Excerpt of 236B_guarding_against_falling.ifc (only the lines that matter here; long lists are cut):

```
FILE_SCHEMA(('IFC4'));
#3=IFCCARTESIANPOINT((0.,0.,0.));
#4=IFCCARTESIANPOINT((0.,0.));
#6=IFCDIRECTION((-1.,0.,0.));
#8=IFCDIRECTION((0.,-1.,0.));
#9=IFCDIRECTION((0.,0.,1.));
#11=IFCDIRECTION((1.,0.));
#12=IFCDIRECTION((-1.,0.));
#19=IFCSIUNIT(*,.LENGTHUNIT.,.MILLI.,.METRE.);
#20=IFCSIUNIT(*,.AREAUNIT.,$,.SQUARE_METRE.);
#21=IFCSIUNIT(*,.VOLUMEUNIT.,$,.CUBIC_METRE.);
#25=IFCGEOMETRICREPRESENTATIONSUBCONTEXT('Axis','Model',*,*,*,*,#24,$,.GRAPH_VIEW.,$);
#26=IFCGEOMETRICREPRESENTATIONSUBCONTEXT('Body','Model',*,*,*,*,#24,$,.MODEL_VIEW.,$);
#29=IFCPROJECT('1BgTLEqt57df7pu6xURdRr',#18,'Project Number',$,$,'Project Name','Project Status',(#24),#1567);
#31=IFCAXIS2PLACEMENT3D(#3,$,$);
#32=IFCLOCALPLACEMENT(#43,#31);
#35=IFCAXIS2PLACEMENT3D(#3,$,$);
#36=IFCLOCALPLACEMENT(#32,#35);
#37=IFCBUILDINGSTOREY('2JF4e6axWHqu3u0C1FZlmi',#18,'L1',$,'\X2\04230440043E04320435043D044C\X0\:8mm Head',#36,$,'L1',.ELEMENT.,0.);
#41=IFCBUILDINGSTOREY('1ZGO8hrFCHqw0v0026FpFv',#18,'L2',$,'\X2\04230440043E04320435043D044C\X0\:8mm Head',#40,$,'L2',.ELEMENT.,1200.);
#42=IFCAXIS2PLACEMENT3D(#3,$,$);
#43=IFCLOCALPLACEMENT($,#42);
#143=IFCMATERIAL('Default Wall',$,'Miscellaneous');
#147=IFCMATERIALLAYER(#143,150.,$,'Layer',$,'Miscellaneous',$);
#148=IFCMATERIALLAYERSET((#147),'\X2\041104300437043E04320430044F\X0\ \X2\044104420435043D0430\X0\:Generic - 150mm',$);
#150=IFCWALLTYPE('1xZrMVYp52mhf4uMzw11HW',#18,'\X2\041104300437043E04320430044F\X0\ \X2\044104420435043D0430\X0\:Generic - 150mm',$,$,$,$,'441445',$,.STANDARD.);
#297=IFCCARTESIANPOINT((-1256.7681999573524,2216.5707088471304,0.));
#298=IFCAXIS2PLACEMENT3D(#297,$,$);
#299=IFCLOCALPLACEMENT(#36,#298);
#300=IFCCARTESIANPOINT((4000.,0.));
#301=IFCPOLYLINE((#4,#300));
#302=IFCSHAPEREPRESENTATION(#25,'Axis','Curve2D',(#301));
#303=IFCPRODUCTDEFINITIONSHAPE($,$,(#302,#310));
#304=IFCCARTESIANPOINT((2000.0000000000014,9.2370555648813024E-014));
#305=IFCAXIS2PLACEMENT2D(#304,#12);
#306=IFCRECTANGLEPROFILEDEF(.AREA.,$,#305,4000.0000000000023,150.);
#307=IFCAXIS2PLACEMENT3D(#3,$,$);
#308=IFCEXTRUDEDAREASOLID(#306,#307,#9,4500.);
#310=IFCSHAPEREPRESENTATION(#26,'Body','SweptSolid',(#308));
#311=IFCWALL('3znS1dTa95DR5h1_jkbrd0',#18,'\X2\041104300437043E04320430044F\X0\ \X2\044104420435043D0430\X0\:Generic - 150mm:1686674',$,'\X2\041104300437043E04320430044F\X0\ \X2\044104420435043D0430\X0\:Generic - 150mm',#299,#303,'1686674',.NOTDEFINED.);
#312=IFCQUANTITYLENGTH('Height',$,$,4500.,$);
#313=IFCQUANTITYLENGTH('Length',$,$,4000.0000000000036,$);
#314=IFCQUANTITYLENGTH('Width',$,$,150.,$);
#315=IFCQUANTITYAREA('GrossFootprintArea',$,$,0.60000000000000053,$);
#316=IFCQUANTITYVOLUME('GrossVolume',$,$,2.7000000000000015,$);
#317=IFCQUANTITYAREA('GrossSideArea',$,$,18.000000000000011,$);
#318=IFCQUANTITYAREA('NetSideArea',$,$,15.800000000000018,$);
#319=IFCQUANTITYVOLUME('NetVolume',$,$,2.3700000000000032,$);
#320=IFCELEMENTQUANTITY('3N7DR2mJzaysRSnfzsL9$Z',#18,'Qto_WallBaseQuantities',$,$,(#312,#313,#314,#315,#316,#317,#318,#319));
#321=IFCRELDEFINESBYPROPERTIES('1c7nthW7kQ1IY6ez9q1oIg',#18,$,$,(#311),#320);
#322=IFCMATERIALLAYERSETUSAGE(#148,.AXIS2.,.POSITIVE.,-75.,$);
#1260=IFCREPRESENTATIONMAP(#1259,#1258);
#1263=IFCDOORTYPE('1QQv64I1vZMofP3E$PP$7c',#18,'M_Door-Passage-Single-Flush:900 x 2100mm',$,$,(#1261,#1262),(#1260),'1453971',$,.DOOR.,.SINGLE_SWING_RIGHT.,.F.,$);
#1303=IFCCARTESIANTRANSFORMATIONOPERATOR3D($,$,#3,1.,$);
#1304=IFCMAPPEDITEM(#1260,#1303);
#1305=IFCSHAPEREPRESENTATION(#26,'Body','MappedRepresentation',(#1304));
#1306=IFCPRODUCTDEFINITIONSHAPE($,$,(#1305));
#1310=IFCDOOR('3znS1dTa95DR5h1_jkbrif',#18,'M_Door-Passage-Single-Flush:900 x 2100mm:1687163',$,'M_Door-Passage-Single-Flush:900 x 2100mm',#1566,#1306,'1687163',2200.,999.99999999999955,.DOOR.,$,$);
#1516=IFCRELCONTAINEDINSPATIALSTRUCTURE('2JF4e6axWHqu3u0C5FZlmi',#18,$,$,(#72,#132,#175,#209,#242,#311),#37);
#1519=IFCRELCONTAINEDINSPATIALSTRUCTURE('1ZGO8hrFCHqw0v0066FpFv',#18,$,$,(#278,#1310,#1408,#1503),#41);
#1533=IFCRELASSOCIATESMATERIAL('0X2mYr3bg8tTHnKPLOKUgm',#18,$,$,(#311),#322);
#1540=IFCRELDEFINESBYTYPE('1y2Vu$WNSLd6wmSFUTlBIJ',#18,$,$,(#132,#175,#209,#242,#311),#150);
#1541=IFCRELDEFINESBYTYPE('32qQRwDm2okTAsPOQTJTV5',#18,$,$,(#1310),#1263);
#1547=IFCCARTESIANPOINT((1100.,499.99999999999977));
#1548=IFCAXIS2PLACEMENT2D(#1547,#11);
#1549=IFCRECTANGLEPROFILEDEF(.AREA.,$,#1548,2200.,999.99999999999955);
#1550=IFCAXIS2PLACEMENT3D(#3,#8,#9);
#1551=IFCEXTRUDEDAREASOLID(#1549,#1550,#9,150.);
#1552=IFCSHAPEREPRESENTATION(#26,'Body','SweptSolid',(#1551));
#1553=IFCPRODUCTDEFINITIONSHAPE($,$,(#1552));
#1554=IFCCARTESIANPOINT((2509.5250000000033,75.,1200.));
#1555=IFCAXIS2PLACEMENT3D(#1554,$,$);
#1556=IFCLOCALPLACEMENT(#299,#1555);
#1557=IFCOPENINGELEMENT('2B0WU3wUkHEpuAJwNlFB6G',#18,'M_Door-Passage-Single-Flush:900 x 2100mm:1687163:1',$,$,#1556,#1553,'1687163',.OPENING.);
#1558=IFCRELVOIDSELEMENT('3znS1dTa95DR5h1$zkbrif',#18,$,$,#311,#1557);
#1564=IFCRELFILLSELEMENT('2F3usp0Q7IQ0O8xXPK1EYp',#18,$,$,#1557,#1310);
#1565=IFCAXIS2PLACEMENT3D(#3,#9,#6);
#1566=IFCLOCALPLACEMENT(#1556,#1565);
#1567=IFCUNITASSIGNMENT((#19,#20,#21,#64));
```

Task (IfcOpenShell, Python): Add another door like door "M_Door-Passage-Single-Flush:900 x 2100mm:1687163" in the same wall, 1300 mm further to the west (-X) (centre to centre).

```python
import ifcopenshell
import ifcopenshell.api.feature
import ifcopenshell.api.geometry
import ifcopenshell.api.pset
import ifcopenshell.api.root
import ifcopenshell.geom
import ifcopenshell.util.element
import ifcopenshell.util.placement
import ifcopenshell.util.shape
import ifcopenshell.util.unit

model = ifcopenshell.open("236B_guarding_against_falling.ifc")
area_scale = ifcopenshell.util.unit.calculate_unit_scale(model, "AREAUNIT")
volume_scale = ifcopenshell.util.unit.calculate_unit_scale(model, "VOLUMEUNIT")
settings = ifcopenshell.geom.settings()


def volume(element):
    """Net volume in cubic metres, openings subtracted."""
    shape = ifcopenshell.geom.create_shape(settings, element)
    return ifcopenshell.util.shape.get_volume(shape.geometry)


def reuse_history(source, copy):
    """copy_class also copies each property set's owner history, people and application; keep the originals."""
    for rel in copy.IsDefinedBy:
        if rel.is_a("IfcRelDefinesByProperties") and (history := rel.RelatingPropertyDefinition.OwnerHistory):
            rel.RelatingPropertyDefinition.OwnerHistory = source.OwnerHistory
            ifcopenshell.util.element.remove_deep2(model, history)


door = model.by_guid("3znS1dTa95DR5h1_jkbrif")
opening = door.FillsVoids[0].RelatingOpeningElement
wall = opening.VoidsElements[0].RelatingBuildingElement
before = volume(wall)
shift = ifcopenshell.util.placement.get_local_placement(wall.ObjectPlacement)[:3, 0] * -1300.0

# copy_class copies the void relationship, type, container and properties, but no geometry.
new_opening = ifcopenshell.api.root.copy_class(model, product=opening)
new_opening.Representation = ifcopenshell.util.element.copy_deep(
    model, opening.Representation, exclude=["IfcGeometricRepresentationContext", "IfcRepresentationMap"]
)
new_opening.Name = "M_Door-Passage-Single-Flush:900 x 2100mm"
new_opening.Tag = None
reuse_history(opening, new_opening)
new_door = ifcopenshell.api.root.copy_class(model, product=door)
new_door.Representation = ifcopenshell.util.element.copy_deep(
    model, door.Representation, exclude=["IfcGeometricRepresentationContext", "IfcRepresentationMap"]
)
new_door.Name = "M_Door-Passage-Single-Flush:900 x 2100mm"
new_door.Tag = None
reuse_history(door, new_door)
ifcopenshell.api.feature.add_filling(model, opening=new_opening, element=new_door)

for old, new in ((opening, new_opening), (door, new_door)):
    matrix = ifcopenshell.util.placement.get_local_placement(old.ObjectPlacement)
    matrix[:3, 3] += shift
    ifcopenshell.api.geometry.edit_object_placement(model, product=new, matrix=matrix, is_si=False)

after = volume(wall)
thickness = 0.15  # wall thickness in metres

# Update the wall's stored quantities.
qto = model.by_id(ifcopenshell.util.element.get_pset(wall, "Qto_WallBaseQuantities", should_inherit=False)["id"])
ifcopenshell.api.pset.edit_qto(model, qto=qto, properties={
    "NetSideArea": after / thickness / area_scale,
    "NetVolume": after / volume_scale,
})

print(f"wall volume {before:.3f} -> {after:.3f} m3")

model.write("236B_guarding_against_falling_v2.ifc")
```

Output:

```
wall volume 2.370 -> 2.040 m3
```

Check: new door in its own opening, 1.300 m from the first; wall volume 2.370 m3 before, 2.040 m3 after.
